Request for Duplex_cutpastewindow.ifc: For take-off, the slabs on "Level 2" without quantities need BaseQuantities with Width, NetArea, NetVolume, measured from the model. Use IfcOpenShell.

First a look at what the model holds.

```python
import ifcopenshell
import ifcopenshell.util.element
import ifcopenshell.util.unit

model = ifcopenshell.open("Duplex_cutpastewindow.ifc")
print(model.schema)
for unit_type in ("LENGTHUNIT", "AREAUNIT", "VOLUMEUNIT"):
    print(unit_type, ifcopenshell.util.unit.calculate_unit_scale(model, unit_type))
storey = next(s for s in model.by_type("IfcBuildingStorey") if s.Name == "Level 2")
slabs = [e for e in ifcopenshell.util.element.get_decomposition(storey) if e.is_a("IfcSlab")]
for e in sorted(slabs, key=lambda e: e.id()):
    print(e.id(), e.is_a(), e.Name, list(ifcopenshell.util.element.get_psets(e, qtos_only=True)), sep=" | ")
```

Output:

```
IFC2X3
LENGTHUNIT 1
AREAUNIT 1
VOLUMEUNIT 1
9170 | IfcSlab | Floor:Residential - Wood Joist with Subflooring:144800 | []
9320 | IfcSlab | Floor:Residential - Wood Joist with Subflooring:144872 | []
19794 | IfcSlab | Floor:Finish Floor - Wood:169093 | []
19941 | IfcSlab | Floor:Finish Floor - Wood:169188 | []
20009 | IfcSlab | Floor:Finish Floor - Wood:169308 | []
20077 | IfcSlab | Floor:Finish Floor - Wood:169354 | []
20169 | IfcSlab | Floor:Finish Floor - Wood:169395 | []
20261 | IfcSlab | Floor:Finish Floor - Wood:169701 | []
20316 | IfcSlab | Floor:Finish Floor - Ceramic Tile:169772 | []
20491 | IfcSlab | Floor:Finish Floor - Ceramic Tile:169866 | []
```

```python
import ifcopenshell
import ifcopenshell.api.pset
import ifcopenshell.geom
import ifcopenshell.util.element
import ifcopenshell.util.shape
import ifcopenshell.util.unit

model = ifcopenshell.open("Duplex_cutpastewindow.ifc")
unit_scale = ifcopenshell.util.unit.calculate_unit_scale(model)
area_scale = ifcopenshell.util.unit.calculate_unit_scale(model, "AREAUNIT")
volume_scale = ifcopenshell.util.unit.calculate_unit_scale(model, "VOLUMEUNIT")
settings = ifcopenshell.geom.settings()

storey = next(s for s in model.by_type("IfcBuildingStorey") if s.Name == "Level 2")
slabs = [e for e in ifcopenshell.util.element.get_decomposition(storey) if e.is_a("IfcSlab")]

for e in sorted(slabs, key=lambda e: e.id()):
    if ifcopenshell.util.element.get_psets(e, qtos_only=True, should_inherit=False):
        continue
    # Geometry comes back in metres, in the element's own axes.
    shape = ifcopenshell.geom.create_shape(settings, e)
    values = {
        "Width": ifcopenshell.util.shape.get_z(shape.geometry) / unit_scale,
        "NetArea": ifcopenshell.util.shape.get_footprint_area(shape.geometry) / area_scale,
        "NetVolume": ifcopenshell.util.shape.get_volume(shape.geometry) / volume_scale,
    }
    qto = ifcopenshell.api.pset.add_qto(model, product=e, name="BaseQuantities")
    ifcopenshell.api.pset.edit_qto(model, qto=qto, properties=values)
    print(e.id(), {k: round(v, 3) for k, v in values.items()})

model.write("Duplex_cutpastewindow_v2.ifc")
```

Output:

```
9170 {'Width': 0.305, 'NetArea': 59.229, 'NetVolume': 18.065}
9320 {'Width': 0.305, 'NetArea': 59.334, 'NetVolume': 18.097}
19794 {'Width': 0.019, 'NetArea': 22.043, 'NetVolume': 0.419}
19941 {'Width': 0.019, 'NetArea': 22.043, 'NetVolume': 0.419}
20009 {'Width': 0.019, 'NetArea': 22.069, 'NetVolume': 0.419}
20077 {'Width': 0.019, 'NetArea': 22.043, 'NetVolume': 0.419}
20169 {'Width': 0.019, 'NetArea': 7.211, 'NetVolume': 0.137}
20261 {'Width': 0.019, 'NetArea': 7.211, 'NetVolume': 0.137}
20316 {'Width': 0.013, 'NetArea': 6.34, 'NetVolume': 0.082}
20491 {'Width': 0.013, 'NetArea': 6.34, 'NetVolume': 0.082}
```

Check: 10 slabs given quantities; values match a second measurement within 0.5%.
